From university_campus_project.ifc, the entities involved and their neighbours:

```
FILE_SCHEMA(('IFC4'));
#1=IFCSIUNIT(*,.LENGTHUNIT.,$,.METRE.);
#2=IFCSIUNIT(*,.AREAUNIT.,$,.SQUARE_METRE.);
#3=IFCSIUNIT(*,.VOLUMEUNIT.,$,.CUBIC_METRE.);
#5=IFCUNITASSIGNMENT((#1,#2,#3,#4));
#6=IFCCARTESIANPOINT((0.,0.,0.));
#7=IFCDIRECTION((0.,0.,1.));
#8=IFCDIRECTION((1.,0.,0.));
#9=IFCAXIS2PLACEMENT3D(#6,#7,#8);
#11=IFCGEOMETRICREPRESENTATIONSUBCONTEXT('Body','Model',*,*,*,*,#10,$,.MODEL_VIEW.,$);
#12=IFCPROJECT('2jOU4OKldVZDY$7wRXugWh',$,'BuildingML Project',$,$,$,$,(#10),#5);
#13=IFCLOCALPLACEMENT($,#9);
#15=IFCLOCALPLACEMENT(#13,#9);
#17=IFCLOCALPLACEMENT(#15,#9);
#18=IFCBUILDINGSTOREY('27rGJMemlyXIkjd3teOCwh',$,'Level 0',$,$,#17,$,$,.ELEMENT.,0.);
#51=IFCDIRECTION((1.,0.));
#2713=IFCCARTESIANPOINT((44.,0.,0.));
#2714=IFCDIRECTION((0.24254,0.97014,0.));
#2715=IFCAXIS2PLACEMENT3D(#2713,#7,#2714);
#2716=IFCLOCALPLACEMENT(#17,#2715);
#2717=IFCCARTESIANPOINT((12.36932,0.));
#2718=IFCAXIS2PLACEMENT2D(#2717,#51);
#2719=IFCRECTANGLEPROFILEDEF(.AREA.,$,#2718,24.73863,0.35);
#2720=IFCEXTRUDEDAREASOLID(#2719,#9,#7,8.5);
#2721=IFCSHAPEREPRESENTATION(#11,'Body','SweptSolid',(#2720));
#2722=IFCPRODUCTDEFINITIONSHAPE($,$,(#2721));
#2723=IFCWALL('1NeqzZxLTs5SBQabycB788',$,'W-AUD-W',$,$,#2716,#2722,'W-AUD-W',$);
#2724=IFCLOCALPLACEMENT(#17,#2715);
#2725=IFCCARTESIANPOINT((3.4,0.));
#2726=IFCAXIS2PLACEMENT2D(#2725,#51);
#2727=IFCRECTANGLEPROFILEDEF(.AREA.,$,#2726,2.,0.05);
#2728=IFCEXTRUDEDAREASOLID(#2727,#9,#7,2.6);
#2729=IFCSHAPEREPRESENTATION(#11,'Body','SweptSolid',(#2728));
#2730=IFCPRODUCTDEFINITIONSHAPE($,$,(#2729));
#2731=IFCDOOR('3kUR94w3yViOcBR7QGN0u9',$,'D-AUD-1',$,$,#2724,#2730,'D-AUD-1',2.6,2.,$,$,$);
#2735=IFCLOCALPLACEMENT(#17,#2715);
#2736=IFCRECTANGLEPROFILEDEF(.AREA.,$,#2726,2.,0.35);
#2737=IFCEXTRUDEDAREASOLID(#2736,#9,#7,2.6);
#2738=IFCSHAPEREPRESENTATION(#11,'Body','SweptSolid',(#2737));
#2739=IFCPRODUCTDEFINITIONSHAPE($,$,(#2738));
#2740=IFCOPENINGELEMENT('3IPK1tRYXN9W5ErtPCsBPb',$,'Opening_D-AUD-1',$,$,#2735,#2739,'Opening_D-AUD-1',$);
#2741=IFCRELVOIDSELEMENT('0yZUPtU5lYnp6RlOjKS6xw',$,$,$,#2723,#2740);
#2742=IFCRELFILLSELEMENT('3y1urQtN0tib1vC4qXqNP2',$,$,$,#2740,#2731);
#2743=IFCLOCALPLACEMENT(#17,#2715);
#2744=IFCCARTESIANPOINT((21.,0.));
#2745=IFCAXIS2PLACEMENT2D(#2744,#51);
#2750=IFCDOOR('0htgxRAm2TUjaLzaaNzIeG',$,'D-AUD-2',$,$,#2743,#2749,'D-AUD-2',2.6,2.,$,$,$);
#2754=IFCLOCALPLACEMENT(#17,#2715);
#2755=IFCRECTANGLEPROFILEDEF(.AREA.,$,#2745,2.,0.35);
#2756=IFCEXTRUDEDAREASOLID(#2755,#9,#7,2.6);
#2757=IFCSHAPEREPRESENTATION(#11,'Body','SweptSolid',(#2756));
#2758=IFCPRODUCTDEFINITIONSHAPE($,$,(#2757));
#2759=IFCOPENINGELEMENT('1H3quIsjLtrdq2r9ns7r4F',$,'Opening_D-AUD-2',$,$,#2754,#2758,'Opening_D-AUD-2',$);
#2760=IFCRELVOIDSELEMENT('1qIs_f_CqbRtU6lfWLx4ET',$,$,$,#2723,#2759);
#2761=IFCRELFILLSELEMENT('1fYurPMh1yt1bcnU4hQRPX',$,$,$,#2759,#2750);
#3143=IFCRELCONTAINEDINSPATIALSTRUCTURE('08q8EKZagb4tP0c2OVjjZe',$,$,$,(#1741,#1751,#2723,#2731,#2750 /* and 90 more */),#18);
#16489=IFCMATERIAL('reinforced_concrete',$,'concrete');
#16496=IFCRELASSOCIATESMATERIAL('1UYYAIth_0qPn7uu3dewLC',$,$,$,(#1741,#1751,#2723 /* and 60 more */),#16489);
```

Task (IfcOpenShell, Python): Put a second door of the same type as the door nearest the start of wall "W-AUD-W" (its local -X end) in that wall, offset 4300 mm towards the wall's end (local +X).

```python
import ifcopenshell
import ifcopenshell.api.feature
import ifcopenshell.api.geometry
import ifcopenshell.api.root
import ifcopenshell.geom
import ifcopenshell.util.element
import ifcopenshell.util.placement
import ifcopenshell.util.shape

model = ifcopenshell.open("university_campus_project.ifc")
settings = ifcopenshell.geom.settings()


def volume(element):
    """Net volume in cubic metres, openings subtracted."""
    shape = ifcopenshell.geom.create_shape(settings, element)
    return ifcopenshell.util.shape.get_volume(shape.geometry)


door = model.by_id(2731)
opening = door.FillsVoids[0].RelatingOpeningElement
wall = opening.VoidsElements[0].RelatingBuildingElement
before = volume(wall)
shift = ifcopenshell.util.placement.get_local_placement(wall.ObjectPlacement)[:3, 0] * 4.3

# copy_class copies the void relationship, type, container and properties, but no geometry.
new_opening = ifcopenshell.api.root.copy_class(model, product=opening)
new_opening.Representation = ifcopenshell.util.element.copy_deep(
    model, opening.Representation, exclude=["IfcGeometricRepresentationContext", "IfcRepresentationMap"]
)
new_opening.Tag = None
new_door = ifcopenshell.api.root.copy_class(model, product=door)
new_door.Representation = ifcopenshell.util.element.copy_deep(
    model, door.Representation, exclude=["IfcGeometricRepresentationContext", "IfcRepresentationMap"]
)
new_door.Tag = None
ifcopenshell.api.feature.add_filling(model, opening=new_opening, element=new_door)

for old, new in ((opening, new_opening), (door, new_door)):
    matrix = ifcopenshell.util.placement.get_local_placement(old.ObjectPlacement)
    matrix[:3, 3] += shift
    ifcopenshell.api.geometry.edit_object_placement(model, product=new, matrix=matrix, is_si=False)

after = volume(wall)

print(f"wall volume {before:.3f} -> {after:.3f} m3")

model.write("university_campus_project_edited.ifc")
```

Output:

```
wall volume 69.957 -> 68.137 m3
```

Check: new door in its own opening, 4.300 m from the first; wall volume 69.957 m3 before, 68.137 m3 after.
